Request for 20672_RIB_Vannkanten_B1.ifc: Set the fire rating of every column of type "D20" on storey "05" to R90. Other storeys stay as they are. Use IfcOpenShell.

First a look at what the model holds.

```python
import ifcopenshell
import ifcopenshell.util.element

model = ifcopenshell.open("20672_RIB_Vannkanten_B1.ifc")
print(model.schema)
storey = next(s for s in model.by_type("IfcBuildingStorey") if s.Name == "05")
columns = [e for e in ifcopenshell.util.element.get_decomposition(storey) if e.is_a("IfcColumn")]
seen = {}
for e in columns:
    element_type = ifcopenshell.util.element.get_type(e)
    key = (element_type.Name if element_type != e and element_type else None, ifcopenshell.util.element.get_pset(e, "Pset_ColumnCommon", "FireRating"))
    seen[key] = seen.get(key, 0) + 1
for (name, value), count in sorted(seen.items(), key=str):
    print(count, "x", name, "|", value)
```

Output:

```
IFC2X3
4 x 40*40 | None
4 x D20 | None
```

```python
import ifcopenshell
import ifcopenshell.api.pset
import ifcopenshell.util.element

model = ifcopenshell.open("20672_RIB_Vannkanten_B1.ifc")

storey = next(s for s in model.by_type("IfcBuildingStorey") if s.Name == "05")
columns = [e for e in ifcopenshell.util.element.get_decomposition(storey) if e.is_a("IfcColumn")]

count = 0
for e in columns:
    element_type = ifcopenshell.util.element.get_type(e)
    if element_type in (None, e) or element_type.Name != "D20":
        continue
    # add_pset returns the element's existing set when there is one.
    pset = ifcopenshell.api.pset.add_pset(model, product=e, name="Pset_ColumnCommon")
    ifcopenshell.api.pset.edit_pset(model, pset=pset, properties={"FireRating": "R90"})
    count += 1

print(count, "columns updated")

model.write("20672_RIB_Vannkanten_B1_updated.ifc")
```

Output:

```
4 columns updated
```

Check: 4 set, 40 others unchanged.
